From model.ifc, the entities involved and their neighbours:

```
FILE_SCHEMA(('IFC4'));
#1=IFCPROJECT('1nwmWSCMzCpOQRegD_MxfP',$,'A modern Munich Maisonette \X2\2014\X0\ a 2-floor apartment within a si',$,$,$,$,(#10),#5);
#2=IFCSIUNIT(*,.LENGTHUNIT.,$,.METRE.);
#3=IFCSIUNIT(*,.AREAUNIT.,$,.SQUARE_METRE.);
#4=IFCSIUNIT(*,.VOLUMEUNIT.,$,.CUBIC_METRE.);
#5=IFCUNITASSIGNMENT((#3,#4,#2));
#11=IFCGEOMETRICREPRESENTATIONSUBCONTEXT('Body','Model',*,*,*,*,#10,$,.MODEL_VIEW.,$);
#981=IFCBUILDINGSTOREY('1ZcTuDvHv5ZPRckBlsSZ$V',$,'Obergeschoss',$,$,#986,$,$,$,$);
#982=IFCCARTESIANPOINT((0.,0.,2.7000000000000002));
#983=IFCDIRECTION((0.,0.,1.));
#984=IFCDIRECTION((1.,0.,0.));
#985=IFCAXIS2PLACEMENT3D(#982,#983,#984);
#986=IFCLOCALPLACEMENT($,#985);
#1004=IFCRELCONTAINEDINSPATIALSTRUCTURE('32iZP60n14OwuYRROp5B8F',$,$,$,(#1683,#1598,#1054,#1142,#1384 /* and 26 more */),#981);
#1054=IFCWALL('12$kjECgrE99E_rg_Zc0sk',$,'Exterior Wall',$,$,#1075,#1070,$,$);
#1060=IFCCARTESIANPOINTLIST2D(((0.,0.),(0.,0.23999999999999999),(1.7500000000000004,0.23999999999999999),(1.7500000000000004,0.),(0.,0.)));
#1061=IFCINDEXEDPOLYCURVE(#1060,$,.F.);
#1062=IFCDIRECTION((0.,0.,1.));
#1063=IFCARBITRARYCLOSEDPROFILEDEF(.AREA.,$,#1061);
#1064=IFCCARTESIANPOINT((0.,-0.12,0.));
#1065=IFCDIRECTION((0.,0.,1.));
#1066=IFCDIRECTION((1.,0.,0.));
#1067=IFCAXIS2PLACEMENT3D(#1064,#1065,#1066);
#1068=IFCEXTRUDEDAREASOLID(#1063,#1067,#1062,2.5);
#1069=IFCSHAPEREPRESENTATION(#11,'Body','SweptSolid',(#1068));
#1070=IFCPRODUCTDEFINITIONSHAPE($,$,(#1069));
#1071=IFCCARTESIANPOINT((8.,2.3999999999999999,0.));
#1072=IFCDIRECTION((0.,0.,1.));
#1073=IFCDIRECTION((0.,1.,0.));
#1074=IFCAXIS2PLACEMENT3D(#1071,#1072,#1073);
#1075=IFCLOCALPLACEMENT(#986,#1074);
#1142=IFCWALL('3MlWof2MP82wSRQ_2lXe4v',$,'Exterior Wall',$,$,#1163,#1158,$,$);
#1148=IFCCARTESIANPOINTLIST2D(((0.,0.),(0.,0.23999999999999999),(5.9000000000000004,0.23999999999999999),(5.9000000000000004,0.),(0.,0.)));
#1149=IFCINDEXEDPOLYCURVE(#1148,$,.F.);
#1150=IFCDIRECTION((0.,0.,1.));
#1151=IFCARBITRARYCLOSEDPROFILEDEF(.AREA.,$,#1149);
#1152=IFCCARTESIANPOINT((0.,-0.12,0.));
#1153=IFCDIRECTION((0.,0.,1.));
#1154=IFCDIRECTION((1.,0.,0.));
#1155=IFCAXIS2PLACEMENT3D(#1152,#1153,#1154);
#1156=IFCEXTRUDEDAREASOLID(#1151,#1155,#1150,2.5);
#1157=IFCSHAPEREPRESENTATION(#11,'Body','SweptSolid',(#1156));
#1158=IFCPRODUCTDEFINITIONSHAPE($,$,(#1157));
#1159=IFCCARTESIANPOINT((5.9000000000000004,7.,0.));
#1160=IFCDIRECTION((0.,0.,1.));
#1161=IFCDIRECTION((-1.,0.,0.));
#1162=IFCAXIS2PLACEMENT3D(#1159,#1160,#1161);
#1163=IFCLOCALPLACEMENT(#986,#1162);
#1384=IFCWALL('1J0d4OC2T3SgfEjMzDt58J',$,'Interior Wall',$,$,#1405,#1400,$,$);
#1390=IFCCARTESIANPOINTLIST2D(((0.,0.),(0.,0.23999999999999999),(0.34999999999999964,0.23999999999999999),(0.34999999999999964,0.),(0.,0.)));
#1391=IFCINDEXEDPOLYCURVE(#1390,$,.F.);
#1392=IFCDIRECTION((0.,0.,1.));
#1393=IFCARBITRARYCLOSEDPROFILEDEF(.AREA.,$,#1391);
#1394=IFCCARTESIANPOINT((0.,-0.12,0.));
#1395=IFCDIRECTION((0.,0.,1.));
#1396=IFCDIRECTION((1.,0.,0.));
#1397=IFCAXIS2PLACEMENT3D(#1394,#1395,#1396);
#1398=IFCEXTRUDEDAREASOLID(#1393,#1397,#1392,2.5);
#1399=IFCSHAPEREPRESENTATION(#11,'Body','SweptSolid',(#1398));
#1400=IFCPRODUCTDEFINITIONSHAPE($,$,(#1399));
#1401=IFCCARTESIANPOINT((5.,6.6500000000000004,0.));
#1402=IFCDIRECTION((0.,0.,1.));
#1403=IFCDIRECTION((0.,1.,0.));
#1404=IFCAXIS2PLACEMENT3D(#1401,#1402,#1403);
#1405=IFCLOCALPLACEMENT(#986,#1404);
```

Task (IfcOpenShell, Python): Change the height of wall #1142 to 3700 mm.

```python
import ifcopenshell
import ifcopenshell.geom
import ifcopenshell.util.representation
import ifcopenshell.util.shape
import ifcopenshell.util.unit

model = ifcopenshell.open("model.ifc")
unit_scale = ifcopenshell.util.unit.calculate_unit_scale(model)
settings = ifcopenshell.geom.settings()


def volume(element):
    """Net volume in cubic metres, openings subtracted."""
    shape = ifcopenshell.geom.create_shape(settings, element)
    return ifcopenshell.util.shape.get_volume(shape.geometry)


wall = model.by_id(1142)
before = volume(wall)

body = ifcopenshell.util.representation.get_representation(wall, "Model", "Body")
solid = body.Items[0]
old_height = solid.Depth
solid.Depth = 3.7 / unit_scale
after = volume(wall)

print(f"height {old_height:g} -> {solid.Depth:g}, volume {before:.3f} -> {after:.3f} m3")

model.write("model_updated.ifc")
```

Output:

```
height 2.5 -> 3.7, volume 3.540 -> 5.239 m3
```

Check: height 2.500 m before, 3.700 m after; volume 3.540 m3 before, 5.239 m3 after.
